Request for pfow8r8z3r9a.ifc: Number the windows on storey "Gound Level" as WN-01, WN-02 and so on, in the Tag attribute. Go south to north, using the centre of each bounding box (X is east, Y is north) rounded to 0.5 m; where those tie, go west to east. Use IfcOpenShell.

First a look at what the model holds.

```python
import ifcopenshell
import ifcopenshell.util.element
import ifcopenshell.util.placement

model = ifcopenshell.open("pfow8r8z3r9a.ifc")
print(model.schema)
storey = next(s for s in model.by_type("IfcBuildingStorey") if s.Name == "Gound Level")
windows = [e for e in ifcopenshell.util.element.get_decomposition(storey) if e.is_a("IfcWindow")]
for e in sorted(windows, key=lambda e: e.id()):
    origin = ifcopenshell.util.placement.get_local_placement(e.ObjectPlacement)[:3, 3]
    print(e.id(), e.Tag, e.Name, origin.round(2) + 0.0, sep=" | ")
```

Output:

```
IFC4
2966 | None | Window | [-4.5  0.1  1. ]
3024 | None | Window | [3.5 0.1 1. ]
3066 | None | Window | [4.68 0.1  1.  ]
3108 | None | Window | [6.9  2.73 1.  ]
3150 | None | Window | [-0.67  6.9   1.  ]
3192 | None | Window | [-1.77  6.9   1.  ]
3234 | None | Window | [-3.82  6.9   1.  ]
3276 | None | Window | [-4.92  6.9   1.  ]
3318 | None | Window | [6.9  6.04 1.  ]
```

```python
import ifcopenshell
import ifcopenshell.geom
import ifcopenshell.util.element
import ifcopenshell.util.shape

model = ifcopenshell.open("pfow8r8z3r9a.ifc")
settings = ifcopenshell.geom.settings()
settings.set("use-world-coords", True)


def centre(element):
    shape = ifcopenshell.geom.create_shape(settings, element)
    return ifcopenshell.util.shape.get_bbox_centroid(shape.geometry)


storey = next(s for s in model.by_type("IfcBuildingStorey") if s.Name == "Gound Level")
windows = [e for e in ifcopenshell.util.element.get_decomposition(storey) if e.is_a("IfcWindow")]

# Insertion points can sit at a corner or the storey origin, so sort by the geometry (in metres).
centres = {e: centre(e) for e in windows}
windows.sort(key=lambda e: (round(centres[e][1] / 0.5), centres[e][0]))

for i, e in enumerate(windows, start=1):
    number = f"WN-{i:02d}"
    e.Tag = number
    print(e.id(), number)

model.write("pfow8r8z3r9a-out.ifc")
```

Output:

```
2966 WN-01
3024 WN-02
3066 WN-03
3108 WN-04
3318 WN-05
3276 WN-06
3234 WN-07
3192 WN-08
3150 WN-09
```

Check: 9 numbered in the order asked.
